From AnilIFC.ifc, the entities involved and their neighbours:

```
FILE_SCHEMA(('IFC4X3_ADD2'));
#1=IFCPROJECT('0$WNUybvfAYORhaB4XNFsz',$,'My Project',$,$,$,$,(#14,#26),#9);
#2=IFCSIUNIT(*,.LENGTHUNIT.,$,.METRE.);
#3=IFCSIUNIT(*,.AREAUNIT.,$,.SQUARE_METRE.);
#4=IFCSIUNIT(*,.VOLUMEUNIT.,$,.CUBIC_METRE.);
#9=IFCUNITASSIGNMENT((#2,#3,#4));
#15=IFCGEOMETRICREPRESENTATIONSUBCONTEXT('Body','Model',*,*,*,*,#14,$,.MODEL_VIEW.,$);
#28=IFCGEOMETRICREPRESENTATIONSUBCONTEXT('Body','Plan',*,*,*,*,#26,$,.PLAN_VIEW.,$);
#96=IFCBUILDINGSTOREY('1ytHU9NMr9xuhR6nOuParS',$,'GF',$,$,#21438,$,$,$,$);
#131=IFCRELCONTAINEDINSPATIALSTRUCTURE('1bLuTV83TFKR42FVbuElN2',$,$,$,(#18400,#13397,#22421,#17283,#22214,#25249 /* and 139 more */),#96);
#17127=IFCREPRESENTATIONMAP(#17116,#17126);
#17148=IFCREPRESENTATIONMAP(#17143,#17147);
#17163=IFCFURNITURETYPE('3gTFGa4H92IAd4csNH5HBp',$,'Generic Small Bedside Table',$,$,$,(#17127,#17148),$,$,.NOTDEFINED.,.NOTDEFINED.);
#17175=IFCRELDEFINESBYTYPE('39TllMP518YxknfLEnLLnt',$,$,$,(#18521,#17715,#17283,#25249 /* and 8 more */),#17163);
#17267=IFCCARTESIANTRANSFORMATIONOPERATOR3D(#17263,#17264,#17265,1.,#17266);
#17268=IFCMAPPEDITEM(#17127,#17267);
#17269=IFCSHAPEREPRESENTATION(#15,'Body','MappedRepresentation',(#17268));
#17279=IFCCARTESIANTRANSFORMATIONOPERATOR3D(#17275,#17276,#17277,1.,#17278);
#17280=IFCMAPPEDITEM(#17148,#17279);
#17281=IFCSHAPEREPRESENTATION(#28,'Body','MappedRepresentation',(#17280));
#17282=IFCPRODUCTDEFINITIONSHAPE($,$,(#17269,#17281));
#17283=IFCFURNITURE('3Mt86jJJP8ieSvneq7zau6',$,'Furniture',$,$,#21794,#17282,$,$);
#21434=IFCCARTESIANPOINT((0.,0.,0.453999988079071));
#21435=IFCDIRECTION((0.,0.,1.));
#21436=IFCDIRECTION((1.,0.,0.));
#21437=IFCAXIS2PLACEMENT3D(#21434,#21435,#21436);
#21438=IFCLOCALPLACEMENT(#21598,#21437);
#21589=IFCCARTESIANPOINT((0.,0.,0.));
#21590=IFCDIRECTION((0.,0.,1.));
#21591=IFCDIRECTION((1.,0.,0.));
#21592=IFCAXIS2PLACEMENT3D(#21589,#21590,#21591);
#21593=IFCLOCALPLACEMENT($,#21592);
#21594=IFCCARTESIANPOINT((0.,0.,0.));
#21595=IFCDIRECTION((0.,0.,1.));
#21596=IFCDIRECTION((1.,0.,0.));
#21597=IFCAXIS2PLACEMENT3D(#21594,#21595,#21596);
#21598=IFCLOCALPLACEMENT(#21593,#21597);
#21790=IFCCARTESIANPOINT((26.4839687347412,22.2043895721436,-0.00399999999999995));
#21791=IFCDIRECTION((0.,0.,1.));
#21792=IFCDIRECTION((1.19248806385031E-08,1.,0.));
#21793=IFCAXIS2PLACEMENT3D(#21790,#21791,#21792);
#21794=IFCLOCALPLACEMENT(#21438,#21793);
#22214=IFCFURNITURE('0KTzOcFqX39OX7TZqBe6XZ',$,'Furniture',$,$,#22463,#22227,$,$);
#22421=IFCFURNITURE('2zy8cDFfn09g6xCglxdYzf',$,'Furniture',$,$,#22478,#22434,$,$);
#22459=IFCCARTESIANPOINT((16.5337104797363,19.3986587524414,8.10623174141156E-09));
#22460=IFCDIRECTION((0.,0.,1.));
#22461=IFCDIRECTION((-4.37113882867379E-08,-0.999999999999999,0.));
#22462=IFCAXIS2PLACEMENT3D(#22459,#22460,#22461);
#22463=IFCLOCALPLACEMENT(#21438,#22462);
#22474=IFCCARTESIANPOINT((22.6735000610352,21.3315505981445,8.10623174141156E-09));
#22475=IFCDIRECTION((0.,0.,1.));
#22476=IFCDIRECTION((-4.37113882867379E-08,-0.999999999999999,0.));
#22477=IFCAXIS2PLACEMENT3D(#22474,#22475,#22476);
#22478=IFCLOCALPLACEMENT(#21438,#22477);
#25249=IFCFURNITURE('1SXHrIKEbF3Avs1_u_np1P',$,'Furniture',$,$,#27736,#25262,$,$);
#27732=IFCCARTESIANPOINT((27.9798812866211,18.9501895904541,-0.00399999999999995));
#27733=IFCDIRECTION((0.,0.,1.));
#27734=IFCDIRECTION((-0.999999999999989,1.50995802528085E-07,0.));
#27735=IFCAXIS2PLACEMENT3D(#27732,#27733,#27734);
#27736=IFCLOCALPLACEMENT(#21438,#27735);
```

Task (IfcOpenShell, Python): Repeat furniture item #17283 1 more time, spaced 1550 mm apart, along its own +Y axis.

```python
import ifcopenshell
import ifcopenshell.api.geometry
import ifcopenshell.api.root
import ifcopenshell.util.element
import ifcopenshell.util.placement

model = ifcopenshell.open("AnilIFC.ifc")

source = model.by_id(17283)
base = ifcopenshell.util.placement.get_local_placement(source.ObjectPlacement)
step = base[:3, 1] * 1.55

for i in range(1, 2):
    copy = ifcopenshell.api.root.copy_class(model, product=source)
    copy.Representation = ifcopenshell.util.element.copy_deep(
        model, source.Representation, exclude=["IfcGeometricRepresentationContext", "IfcRepresentationMap"]
    )
    matrix = base.copy()
    matrix[:3, 3] += i * step
    print("added at", matrix[:3, 3].round(3) + 0.0)
    ifcopenshell.api.geometry.edit_object_placement(model, product=copy, matrix=matrix, is_si=False)

model.write("AnilIFC_rev.ifc")
```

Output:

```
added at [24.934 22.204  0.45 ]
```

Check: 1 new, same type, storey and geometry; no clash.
